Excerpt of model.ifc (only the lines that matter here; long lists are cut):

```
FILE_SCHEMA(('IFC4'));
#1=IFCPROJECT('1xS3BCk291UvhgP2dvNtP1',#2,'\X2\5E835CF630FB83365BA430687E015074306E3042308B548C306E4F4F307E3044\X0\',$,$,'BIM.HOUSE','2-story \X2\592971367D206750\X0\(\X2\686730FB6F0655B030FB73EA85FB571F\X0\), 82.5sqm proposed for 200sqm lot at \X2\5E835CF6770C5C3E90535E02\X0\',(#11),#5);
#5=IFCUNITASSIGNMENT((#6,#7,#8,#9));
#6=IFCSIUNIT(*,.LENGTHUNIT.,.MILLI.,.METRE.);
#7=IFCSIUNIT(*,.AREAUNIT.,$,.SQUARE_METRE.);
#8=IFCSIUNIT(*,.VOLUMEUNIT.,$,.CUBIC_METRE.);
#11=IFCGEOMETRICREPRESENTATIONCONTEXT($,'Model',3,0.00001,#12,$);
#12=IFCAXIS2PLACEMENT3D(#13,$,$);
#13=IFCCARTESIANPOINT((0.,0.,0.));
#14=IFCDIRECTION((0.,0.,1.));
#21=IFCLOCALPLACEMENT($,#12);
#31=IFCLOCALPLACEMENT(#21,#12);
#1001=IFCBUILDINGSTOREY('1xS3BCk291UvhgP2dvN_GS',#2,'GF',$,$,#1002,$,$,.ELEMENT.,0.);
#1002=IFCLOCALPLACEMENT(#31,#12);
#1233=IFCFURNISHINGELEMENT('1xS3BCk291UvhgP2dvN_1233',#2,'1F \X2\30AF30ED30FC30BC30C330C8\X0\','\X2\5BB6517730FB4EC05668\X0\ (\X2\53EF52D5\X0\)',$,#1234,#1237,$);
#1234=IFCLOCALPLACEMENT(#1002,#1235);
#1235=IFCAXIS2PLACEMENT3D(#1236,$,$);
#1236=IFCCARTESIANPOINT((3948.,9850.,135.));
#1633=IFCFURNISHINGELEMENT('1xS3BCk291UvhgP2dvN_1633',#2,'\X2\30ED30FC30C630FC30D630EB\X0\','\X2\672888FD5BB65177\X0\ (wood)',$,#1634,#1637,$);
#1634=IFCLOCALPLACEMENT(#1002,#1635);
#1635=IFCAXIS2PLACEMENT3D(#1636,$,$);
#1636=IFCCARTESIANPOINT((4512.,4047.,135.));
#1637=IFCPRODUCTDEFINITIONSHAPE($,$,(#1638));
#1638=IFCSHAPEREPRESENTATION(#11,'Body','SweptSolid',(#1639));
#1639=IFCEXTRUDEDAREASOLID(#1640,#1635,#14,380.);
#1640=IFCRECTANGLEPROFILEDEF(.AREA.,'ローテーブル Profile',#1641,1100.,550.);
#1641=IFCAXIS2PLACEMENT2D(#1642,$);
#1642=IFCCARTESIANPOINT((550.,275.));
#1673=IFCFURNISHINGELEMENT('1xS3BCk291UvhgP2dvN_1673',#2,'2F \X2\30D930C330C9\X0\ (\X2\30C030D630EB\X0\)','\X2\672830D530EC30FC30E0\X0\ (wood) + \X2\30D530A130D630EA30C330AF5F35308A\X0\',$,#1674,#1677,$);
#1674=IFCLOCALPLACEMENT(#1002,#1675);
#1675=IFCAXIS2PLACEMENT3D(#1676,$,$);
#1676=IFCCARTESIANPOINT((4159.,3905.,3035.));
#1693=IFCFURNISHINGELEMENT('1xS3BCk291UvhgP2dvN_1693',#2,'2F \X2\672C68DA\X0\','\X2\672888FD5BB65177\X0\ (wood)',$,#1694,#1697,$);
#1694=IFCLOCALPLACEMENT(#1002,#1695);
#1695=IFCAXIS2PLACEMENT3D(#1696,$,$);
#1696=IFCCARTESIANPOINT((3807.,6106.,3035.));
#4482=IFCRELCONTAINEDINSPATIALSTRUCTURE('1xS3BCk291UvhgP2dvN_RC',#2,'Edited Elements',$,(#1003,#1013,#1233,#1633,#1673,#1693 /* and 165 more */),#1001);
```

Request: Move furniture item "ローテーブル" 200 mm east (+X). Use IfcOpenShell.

```python
import ifcopenshell
import ifcopenshell.api.geometry
import ifcopenshell.util.placement

model = ifcopenshell.open("model.ifc")

item = model.by_id(1633)
matrix = ifcopenshell.util.placement.get_local_placement(item.ObjectPlacement)
matrix[0, 3] += 200.0
ifcopenshell.api.geometry.edit_object_placement(model, product=item, matrix=matrix, is_si=False)

print(ifcopenshell.util.placement.get_local_placement(item.ObjectPlacement).round(3) + 0.0)

model.write("model_updated.ifc")
```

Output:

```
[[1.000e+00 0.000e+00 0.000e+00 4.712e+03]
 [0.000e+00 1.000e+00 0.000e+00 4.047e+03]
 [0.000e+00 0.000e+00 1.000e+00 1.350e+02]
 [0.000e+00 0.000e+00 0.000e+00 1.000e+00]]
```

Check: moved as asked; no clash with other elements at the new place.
